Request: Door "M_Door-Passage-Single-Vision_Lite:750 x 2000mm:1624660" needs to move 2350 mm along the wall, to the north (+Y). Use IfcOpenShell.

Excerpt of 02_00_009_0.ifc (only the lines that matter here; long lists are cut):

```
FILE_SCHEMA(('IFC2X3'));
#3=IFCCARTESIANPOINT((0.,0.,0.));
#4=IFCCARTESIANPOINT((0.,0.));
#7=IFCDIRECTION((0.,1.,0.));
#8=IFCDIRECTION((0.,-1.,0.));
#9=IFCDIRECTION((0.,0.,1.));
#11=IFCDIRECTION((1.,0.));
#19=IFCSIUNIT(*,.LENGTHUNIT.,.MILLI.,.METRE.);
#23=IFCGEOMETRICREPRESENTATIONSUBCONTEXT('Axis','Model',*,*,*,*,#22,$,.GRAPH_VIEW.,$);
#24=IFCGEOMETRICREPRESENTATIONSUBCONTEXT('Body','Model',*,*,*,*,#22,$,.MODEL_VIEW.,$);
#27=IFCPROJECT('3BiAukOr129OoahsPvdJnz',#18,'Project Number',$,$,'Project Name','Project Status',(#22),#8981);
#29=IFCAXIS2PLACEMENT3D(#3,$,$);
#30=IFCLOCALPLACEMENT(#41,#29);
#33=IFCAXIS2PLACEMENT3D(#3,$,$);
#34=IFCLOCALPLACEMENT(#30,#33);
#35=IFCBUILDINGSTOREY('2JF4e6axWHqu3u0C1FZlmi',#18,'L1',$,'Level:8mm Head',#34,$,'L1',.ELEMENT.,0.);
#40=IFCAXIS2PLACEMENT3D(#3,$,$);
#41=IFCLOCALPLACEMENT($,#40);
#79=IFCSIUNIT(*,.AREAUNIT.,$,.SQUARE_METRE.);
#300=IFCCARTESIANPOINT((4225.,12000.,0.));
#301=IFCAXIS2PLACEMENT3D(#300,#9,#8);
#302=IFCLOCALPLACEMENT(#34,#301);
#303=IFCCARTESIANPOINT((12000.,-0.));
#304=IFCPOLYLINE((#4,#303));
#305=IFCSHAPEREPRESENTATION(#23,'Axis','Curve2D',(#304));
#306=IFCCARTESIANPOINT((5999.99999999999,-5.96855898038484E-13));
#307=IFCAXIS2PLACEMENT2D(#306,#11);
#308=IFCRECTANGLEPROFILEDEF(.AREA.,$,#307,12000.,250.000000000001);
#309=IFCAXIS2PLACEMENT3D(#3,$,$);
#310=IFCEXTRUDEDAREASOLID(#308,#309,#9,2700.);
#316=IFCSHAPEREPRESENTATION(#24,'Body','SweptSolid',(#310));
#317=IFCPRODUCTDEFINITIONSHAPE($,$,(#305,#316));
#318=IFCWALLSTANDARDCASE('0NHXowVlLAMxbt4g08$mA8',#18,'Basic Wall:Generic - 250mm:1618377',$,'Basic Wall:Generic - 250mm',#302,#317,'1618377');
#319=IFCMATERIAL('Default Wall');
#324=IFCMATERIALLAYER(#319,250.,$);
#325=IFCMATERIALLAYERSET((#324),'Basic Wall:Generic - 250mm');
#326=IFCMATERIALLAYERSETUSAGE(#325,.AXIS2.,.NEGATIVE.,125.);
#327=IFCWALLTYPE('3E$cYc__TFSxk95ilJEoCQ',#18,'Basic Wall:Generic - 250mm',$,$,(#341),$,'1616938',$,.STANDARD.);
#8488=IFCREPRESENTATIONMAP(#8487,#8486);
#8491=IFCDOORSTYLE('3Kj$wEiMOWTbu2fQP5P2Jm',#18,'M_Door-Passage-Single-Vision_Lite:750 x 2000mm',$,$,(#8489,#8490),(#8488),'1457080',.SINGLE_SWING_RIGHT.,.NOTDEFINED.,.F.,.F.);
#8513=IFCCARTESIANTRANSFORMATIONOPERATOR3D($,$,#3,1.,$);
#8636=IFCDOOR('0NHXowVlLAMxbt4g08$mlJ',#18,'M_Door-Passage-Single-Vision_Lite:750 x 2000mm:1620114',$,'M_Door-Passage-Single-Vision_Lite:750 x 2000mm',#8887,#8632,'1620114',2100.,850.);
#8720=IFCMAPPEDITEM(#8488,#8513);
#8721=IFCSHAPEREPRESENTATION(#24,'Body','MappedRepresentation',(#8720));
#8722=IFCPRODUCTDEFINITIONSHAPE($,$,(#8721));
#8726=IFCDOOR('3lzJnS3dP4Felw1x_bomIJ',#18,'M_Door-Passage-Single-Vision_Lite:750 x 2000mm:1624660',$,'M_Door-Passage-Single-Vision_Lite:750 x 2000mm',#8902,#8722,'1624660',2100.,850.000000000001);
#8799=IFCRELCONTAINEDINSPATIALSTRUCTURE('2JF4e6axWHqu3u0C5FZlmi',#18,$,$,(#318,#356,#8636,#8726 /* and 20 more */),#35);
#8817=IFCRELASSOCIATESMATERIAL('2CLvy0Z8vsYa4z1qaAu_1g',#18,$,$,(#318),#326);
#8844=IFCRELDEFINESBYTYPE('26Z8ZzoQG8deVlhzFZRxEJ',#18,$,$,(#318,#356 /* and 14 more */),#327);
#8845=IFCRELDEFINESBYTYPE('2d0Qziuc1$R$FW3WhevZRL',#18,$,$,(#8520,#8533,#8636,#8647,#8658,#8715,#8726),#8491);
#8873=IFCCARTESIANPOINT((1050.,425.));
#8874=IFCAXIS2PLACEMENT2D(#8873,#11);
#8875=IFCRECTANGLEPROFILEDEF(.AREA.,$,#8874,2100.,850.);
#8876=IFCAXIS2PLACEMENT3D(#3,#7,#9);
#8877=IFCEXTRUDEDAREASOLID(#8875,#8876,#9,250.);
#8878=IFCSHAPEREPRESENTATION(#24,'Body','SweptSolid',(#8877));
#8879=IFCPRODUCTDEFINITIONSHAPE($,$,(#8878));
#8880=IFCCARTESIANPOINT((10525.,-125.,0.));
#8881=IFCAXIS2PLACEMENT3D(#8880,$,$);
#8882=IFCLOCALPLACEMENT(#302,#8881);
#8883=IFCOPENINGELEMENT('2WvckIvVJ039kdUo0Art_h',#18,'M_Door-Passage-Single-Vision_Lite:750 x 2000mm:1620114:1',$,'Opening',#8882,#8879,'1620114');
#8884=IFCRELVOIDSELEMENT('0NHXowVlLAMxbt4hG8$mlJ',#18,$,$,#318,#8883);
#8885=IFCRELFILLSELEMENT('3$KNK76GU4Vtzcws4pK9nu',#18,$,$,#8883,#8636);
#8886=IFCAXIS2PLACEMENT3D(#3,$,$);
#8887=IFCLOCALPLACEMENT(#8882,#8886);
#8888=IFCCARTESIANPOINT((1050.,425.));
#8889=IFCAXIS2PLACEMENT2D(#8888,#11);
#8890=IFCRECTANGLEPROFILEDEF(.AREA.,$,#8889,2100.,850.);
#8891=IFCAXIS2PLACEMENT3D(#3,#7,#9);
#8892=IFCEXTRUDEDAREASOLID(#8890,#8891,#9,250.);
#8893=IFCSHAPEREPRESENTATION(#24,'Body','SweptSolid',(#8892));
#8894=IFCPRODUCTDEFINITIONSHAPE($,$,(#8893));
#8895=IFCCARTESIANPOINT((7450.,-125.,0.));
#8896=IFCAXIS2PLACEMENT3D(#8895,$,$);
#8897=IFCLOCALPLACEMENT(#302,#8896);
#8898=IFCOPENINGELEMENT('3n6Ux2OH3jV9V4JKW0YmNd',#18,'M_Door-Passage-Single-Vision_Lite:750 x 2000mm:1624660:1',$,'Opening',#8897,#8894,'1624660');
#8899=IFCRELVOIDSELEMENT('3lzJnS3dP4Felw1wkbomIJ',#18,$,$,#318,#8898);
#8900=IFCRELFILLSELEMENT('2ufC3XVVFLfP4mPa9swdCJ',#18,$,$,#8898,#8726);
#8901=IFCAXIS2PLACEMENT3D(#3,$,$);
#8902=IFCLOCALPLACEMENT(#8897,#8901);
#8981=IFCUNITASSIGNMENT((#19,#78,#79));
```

```python
import ifcopenshell
import ifcopenshell.api.geometry
import ifcopenshell.util.placement
import ifcopenshell.util.unit

model = ifcopenshell.open("02_00_009_0.ifc")
unit_scale = ifcopenshell.util.unit.calculate_unit_scale(model)

door = model.by_guid("3lzJnS3dP4Felw1x_bomIJ")
opening = door.FillsVoids[0].RelatingOpeningElement
wall = opening.VoidsElements[0].RelatingBuildingElement

wall_matrix = ifcopenshell.util.placement.get_local_placement(wall.ObjectPlacement)
shift = wall_matrix[:3, 0] * -2.35 / unit_scale
before = ifcopenshell.util.placement.get_local_placement(door.ObjectPlacement)[:3, 3].copy()

# The door is placed relative to its opening, so it follows when the opening moves.
matrix = ifcopenshell.util.placement.get_local_placement(opening.ObjectPlacement)
matrix[:3, 3] += shift
ifcopenshell.api.geometry.edit_object_placement(
    model, product=opening, matrix=matrix, is_si=False, should_transform_children=True
)

after = ifcopenshell.util.placement.get_local_placement(door.ObjectPlacement)[:3, 3]
print("door moved by", (after - before).round(3) + 0.0)

model.write("02_00_009_0_edited.ifc")
```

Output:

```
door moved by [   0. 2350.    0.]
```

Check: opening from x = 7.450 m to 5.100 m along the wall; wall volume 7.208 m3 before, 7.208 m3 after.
